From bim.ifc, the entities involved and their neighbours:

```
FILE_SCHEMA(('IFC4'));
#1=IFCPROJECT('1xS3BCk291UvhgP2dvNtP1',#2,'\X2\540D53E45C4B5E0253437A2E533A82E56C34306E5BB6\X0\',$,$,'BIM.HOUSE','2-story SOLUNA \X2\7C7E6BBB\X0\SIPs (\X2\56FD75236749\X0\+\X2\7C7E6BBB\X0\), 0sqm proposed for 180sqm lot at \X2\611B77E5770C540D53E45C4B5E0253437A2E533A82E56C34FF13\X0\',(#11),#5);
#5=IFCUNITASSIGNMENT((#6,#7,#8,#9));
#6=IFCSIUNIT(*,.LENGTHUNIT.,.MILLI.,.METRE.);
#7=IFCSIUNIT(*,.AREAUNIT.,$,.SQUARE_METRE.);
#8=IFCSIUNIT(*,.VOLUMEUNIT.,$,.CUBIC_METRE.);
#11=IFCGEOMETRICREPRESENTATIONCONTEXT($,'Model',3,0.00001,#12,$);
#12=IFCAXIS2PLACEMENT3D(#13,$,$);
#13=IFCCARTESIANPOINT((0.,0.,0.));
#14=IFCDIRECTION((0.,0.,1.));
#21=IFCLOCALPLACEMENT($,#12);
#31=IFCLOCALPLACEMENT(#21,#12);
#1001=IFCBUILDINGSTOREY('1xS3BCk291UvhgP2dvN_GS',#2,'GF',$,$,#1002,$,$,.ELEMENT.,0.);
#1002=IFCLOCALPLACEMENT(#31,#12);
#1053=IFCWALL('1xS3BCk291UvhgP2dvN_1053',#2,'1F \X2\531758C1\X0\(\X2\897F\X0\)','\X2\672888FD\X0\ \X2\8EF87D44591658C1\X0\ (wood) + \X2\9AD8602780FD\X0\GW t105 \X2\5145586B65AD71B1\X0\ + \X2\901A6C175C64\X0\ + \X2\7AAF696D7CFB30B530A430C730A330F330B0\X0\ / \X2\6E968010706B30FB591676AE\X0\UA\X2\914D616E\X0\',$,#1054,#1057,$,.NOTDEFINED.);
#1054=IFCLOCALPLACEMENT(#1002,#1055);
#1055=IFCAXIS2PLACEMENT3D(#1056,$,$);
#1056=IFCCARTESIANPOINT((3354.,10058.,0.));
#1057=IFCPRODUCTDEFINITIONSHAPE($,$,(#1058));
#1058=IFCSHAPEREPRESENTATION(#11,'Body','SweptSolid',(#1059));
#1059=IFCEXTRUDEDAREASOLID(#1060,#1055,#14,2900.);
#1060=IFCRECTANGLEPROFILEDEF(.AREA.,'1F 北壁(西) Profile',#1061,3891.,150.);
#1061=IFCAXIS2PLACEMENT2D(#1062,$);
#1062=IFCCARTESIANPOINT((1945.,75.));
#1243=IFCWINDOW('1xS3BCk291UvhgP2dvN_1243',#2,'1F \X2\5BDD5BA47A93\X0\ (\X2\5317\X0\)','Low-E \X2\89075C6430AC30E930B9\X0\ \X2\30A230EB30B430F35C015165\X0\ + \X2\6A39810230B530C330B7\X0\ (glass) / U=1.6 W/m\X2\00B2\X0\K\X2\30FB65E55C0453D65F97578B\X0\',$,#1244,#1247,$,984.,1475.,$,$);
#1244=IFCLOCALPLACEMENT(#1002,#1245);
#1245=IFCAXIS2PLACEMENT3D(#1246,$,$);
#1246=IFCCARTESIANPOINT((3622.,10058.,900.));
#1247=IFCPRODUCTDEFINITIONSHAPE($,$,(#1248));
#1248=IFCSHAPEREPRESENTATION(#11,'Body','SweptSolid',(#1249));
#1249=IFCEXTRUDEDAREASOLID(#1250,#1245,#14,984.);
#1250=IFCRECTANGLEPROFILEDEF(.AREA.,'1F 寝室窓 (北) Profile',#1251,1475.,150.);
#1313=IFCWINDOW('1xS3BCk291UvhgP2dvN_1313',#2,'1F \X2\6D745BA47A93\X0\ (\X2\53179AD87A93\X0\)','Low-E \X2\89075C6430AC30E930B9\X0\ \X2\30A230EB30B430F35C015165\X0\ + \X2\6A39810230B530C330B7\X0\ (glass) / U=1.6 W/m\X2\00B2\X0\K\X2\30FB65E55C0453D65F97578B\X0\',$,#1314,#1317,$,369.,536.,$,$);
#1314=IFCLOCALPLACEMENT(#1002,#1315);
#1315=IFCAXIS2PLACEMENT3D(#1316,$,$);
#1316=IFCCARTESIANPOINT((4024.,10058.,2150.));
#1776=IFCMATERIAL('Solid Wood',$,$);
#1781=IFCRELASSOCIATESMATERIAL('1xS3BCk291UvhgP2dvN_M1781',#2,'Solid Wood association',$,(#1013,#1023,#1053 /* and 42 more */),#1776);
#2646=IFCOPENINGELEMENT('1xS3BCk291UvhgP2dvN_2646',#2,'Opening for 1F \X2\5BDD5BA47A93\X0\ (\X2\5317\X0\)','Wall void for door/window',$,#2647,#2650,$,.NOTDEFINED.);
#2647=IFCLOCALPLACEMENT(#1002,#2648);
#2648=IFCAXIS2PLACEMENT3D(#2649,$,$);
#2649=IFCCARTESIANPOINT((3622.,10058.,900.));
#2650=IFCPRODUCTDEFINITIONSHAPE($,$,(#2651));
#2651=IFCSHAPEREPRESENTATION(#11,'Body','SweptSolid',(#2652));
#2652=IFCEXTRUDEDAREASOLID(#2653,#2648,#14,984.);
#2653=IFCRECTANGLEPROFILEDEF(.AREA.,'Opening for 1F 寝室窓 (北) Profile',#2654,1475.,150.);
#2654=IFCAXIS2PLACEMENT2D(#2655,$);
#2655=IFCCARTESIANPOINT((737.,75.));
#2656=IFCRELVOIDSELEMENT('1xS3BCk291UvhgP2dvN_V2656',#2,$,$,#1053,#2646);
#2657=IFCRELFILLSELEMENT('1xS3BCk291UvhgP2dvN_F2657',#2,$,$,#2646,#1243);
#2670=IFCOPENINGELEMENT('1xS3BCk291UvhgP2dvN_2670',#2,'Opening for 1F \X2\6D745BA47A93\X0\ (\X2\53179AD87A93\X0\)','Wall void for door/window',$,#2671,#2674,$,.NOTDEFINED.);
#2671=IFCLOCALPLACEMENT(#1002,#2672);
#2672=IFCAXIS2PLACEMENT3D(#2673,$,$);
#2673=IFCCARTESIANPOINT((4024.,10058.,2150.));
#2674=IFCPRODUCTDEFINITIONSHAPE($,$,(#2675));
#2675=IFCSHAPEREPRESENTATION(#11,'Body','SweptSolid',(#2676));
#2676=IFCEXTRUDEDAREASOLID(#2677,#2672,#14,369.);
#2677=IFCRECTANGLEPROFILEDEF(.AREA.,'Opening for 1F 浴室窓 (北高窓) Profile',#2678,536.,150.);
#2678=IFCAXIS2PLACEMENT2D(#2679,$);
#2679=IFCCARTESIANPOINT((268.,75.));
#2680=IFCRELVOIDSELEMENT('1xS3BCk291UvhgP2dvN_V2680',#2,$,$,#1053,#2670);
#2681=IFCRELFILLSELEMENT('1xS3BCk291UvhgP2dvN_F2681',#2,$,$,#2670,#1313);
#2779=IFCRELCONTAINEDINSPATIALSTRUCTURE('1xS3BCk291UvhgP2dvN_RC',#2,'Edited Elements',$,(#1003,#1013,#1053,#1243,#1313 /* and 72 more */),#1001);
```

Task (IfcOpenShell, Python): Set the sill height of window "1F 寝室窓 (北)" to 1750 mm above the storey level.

```python
import numpy as np
import ifcopenshell
import ifcopenshell.api.geometry
import ifcopenshell.geom
import ifcopenshell.util.element
import ifcopenshell.util.placement
import ifcopenshell.util.shape
import ifcopenshell.util.unit

model = ifcopenshell.open("bim.ifc")
unit_scale = ifcopenshell.util.unit.calculate_unit_scale(model)

window = model.by_guid("1xS3BCk291UvhgP2dvN_1243")
opening = window.FillsVoids[0].RelatingOpeningElement
storey = ifcopenshell.util.element.get_container(window, ifc_class="IfcBuildingStorey")
level = ifcopenshell.util.placement.get_local_placement(storey.ObjectPlacement)[2, 3]

# The opening's origin need not be at the sill, so measure its lowest point.
shape = ifcopenshell.geom.create_shape(ifcopenshell.geom.settings(), opening)
bottom = ifcopenshell.util.shape.get_shape_bottom_elevation(shape, shape.geometry) / unit_scale
dz = level + 1750.0 - bottom

shift = np.array([0.0, 0.0, dz])
# The window is not placed relative to its opening, so move both.
for product in (opening, window):
    matrix = ifcopenshell.util.placement.get_local_placement(product.ObjectPlacement)
    matrix[:3, 3] += shift
    ifcopenshell.api.geometry.edit_object_placement(model, product=product, matrix=matrix, is_si=False)

print(f"moved by {dz * unit_scale:+.3f} m")

model.write("bim_updated.ifc")
```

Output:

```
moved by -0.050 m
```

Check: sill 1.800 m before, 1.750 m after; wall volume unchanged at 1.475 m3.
